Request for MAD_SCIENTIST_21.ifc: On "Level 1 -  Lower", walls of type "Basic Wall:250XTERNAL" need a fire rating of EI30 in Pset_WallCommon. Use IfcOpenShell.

First a look at what the model holds.

```python
import ifcopenshell
import ifcopenshell.util.element

model = ifcopenshell.open("MAD_SCIENTIST_21.ifc")
print(model.schema)
storey = next(s for s in model.by_type("IfcBuildingStorey") if s.Name == "Level 1 -  Lower")
walls = [e for e in ifcopenshell.util.element.get_decomposition(storey) if e.is_a("IfcWall")]
seen = {}
for e in walls:
    element_type = ifcopenshell.util.element.get_type(e)
    key = (element_type.Name if element_type != e and element_type else None, ifcopenshell.util.element.get_pset(e, "Pset_WallCommon", "FireRating"))
    seen[key] = seen.get(key, 0) + 1
for (name, value), count in sorted(seen.items(), key=str):
    print(count, "x", name, "|", value)
```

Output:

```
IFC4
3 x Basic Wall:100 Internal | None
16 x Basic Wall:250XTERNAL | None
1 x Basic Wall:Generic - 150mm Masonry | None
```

```python
import ifcopenshell
import ifcopenshell.api.pset
import ifcopenshell.util.element

model = ifcopenshell.open("MAD_SCIENTIST_21.ifc")

storey = next(s for s in model.by_type("IfcBuildingStorey") if s.Name == "Level 1 -  Lower")
walls = [e for e in ifcopenshell.util.element.get_decomposition(storey) if e.is_a("IfcWall")]

count = 0
for e in walls:
    element_type = ifcopenshell.util.element.get_type(e)
    if element_type in (None, e) or element_type.Name != "Basic Wall:250XTERNAL":
        continue
    # add_pset returns the element's existing set when there is one.
    pset = ifcopenshell.api.pset.add_pset(model, product=e, name="Pset_WallCommon")
    ifcopenshell.api.pset.edit_pset(model, pset=pset, properties={"FireRating": "EI30"})
    count += 1

print(count, "walls updated")

model.write("MAD_SCIENTIST_21_updated.ifc")
```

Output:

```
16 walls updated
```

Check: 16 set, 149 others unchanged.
